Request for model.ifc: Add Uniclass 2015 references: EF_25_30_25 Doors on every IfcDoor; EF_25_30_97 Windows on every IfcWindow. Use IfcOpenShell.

First a look at what the model holds.

```python
import ifcopenshell

model = ifcopenshell.open("model.ifc")
print(model.schema)
print("classifications:", [c.Name for c in model.by_type("IfcClassification")])
for ifc_class in ("IfcDoor", "IfcRoof", "IfcStair", "IfcWall", "IfcWindow"):
    print(ifc_class, len(model.by_type(ifc_class)))
```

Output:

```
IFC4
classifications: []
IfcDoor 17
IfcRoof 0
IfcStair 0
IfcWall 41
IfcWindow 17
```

```python
import ifcopenshell
import ifcopenshell.api.classification

model = ifcopenshell.open("model.ifc")

system = ifcopenshell.api.classification.add_classification(model, classification="Uniclass 2015")

codes = {
    "IfcDoor": ("EF_25_30_25", "Doors"),
    "IfcWindow": ("EF_25_30_97", "Windows"),
}
for ifc_class, (code, name) in codes.items():
    products = model.by_type(ifc_class)
    ifcopenshell.api.classification.add_reference(
        model, products=products, classification=system, identification=code, name=name
    )
    print(code, len(products))

model.write("model-out.ifc")
```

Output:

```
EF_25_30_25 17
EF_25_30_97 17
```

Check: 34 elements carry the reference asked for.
